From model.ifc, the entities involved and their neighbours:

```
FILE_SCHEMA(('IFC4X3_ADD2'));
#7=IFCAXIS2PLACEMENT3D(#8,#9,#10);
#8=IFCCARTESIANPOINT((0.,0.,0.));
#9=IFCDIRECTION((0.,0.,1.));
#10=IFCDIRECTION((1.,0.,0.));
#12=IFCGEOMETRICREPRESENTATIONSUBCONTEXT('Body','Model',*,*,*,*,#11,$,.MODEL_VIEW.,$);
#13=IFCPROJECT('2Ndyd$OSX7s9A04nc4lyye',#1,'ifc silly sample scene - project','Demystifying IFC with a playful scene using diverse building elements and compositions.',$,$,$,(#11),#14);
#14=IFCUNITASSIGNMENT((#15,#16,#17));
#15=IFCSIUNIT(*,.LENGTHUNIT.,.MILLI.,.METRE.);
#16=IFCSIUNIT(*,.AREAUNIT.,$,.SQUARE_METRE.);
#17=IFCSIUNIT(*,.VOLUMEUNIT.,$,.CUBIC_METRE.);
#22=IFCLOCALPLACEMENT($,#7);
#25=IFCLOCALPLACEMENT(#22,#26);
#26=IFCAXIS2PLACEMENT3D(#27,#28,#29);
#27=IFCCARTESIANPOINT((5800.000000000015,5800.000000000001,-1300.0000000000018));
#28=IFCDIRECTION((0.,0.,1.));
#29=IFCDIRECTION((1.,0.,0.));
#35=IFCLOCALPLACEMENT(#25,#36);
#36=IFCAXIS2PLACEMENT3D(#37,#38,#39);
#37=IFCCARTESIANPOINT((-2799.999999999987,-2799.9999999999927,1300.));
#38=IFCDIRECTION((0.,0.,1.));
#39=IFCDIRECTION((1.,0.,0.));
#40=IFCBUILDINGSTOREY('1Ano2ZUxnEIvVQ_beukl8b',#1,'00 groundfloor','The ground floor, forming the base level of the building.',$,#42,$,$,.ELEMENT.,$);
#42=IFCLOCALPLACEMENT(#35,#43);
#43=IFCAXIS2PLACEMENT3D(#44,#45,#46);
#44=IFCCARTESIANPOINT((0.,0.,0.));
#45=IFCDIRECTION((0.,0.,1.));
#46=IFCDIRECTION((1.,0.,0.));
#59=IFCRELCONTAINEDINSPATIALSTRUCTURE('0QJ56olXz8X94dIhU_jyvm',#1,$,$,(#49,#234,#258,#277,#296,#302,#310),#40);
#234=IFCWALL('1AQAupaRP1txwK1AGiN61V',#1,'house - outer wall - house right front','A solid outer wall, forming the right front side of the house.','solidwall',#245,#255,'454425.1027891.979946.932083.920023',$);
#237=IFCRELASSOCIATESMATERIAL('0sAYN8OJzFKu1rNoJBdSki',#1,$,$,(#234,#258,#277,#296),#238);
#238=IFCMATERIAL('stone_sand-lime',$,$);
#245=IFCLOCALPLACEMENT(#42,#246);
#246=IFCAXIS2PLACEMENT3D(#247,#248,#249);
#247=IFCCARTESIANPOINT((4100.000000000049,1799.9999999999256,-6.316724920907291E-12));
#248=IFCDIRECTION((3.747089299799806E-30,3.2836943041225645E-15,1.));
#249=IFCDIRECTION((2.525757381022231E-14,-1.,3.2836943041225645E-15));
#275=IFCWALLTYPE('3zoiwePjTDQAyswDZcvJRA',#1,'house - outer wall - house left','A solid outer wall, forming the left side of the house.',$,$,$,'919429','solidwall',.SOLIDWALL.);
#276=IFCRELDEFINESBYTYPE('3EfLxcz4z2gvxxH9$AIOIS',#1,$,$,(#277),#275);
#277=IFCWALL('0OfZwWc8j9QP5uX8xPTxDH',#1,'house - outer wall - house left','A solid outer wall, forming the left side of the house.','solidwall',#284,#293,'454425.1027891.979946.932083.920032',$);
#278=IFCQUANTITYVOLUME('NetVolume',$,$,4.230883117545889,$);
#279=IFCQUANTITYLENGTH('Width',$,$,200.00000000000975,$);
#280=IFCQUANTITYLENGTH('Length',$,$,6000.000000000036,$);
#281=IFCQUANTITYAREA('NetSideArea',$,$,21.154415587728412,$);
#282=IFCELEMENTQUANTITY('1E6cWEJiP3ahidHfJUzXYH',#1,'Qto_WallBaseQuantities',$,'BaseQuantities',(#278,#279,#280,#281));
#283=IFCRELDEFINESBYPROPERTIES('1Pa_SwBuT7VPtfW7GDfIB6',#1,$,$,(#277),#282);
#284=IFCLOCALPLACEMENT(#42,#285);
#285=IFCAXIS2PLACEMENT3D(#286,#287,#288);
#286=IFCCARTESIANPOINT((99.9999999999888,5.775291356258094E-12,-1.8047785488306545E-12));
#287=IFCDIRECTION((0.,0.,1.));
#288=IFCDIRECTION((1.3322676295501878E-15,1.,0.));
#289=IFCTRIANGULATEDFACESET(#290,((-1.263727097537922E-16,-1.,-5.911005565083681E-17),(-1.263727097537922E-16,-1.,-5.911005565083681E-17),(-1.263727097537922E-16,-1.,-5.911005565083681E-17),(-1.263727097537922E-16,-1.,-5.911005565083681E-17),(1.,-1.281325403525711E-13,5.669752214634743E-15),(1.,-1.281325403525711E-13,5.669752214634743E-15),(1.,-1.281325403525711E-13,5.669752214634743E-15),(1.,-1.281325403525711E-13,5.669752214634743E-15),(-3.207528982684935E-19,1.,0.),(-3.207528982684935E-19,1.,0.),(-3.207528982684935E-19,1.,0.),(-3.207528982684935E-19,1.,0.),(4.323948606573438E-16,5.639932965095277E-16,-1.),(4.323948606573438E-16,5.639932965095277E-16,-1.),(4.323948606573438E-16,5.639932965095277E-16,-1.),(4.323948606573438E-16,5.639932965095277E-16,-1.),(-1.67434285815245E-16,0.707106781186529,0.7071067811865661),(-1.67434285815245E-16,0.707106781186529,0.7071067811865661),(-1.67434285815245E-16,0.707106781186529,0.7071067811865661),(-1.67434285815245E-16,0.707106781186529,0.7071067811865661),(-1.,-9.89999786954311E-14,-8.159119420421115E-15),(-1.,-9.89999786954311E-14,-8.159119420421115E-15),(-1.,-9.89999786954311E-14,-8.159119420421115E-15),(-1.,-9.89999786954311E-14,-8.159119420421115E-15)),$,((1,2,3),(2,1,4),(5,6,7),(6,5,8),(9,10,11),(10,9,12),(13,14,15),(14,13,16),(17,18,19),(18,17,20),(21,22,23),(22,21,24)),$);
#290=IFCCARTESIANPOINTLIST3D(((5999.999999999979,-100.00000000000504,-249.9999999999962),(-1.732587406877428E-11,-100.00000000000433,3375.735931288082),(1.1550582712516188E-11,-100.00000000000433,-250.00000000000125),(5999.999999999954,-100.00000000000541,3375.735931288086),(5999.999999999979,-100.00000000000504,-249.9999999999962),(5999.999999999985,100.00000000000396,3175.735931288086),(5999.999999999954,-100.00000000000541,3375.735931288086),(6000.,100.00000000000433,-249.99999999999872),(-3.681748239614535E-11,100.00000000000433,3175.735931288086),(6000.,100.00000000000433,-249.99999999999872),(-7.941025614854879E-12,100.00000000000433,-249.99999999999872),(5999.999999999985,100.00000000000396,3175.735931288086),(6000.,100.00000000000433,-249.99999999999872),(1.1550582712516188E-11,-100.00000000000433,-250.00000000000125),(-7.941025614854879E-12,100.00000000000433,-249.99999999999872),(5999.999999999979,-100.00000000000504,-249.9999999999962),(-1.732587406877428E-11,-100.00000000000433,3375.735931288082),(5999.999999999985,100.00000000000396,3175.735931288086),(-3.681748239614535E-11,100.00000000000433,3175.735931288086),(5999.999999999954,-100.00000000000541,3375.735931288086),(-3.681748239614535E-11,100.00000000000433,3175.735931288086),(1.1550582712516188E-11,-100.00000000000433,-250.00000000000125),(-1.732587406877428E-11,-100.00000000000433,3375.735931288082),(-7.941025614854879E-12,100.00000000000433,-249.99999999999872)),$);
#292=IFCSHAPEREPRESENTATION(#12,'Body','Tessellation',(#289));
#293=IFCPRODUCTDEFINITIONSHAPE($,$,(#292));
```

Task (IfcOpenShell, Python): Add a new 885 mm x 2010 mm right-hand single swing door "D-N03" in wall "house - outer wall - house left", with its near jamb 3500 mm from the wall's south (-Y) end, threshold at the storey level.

```python
import numpy as np
import ifcopenshell
import ifcopenshell.api.feature
import ifcopenshell.api.geometry
import ifcopenshell.api.pset
import ifcopenshell.api.root
import ifcopenshell.api.spatial
import ifcopenshell.geom
import ifcopenshell.util.element
import ifcopenshell.util.placement
import ifcopenshell.util.representation
import ifcopenshell.util.shape
import ifcopenshell.util.unit

model = ifcopenshell.open("model.ifc")
unit_scale = ifcopenshell.util.unit.calculate_unit_scale(model)
area_scale = ifcopenshell.util.unit.calculate_unit_scale(model, "AREAUNIT")
volume_scale = ifcopenshell.util.unit.calculate_unit_scale(model, "VOLUMEUNIT")
settings = ifcopenshell.geom.settings()


def volume(element):
    """Net volume in cubic metres, openings subtracted."""
    shape = ifcopenshell.geom.create_shape(settings, element)
    return ifcopenshell.util.shape.get_volume(shape.geometry)


wall = model.by_guid("0OfZwWc8j9QP5uX8xPTxDH")
storey = ifcopenshell.util.element.get_container(wall, ifc_class="IfcBuildingStorey")
context = ifcopenshell.util.representation.get_context(model, "Model", "Body", "MODEL_VIEW")
before = volume(wall)

width, height, from_end, sill = 0.885, 2.01, 3.5, 0.0  # metres

# The wall runs along its own X axis, and the end named is its -X end.
wall_shape = ifcopenshell.geom.create_shape(settings, wall)
x, y, z = ifcopenshell.util.shape.get_vertices(wall_shape.geometry).T
start = x.min() + from_end
face, thickness = float(y.min()), float(y.max() - y.min())
wall_matrix = ifcopenshell.util.placement.get_local_placement(wall.ObjectPlacement)
level = ifcopenshell.util.placement.get_local_placement(storey.ObjectPlacement)[2, 3]


def in_wall(x, y):
    """Placement at x, y metres in the wall's axes, at sill height."""
    matrix = wall_matrix.copy()
    matrix[:, 3] = wall_matrix @ np.array([x / unit_scale, y / unit_scale, 0.0, 1.0])
    matrix[2, 3] = level + sill / unit_scale
    return matrix


# Opening: a box that overshoots both wall faces by 50 mm.
opening = ifcopenshell.api.root.create_entity(model, ifc_class="IfcOpeningElement", predefined_type="OPENING")
box = ifcopenshell.api.geometry.add_wall_representation(
    model, context=context, length=width, height=height, thickness=thickness + 0.1
)
ifcopenshell.api.geometry.assign_representation(model, product=opening, representation=box)
ifcopenshell.api.geometry.edit_object_placement(model, product=opening, matrix=in_wall(start, face - 0.05), is_si=False)
ifcopenshell.api.feature.add_feature(model, feature=opening, element=wall)

door = ifcopenshell.api.root.create_entity(model, ifc_class="IfcDoor", name="D-N03", predefined_type="DOOR")
door.OverallWidth, door.OverallHeight = width / unit_scale, height / unit_scale
door.OperationType = "SINGLE_SWING_RIGHT"
body = ifcopenshell.api.geometry.add_door_representation(
    model,
    context=context,
    overall_width=door.OverallWidth,
    overall_height=door.OverallHeight,
    operation_type="SINGLE_SWING_RIGHT",
    lining_properties={"LiningDepth": thickness / unit_scale, "ThresholdDepth": thickness / unit_scale},
)
ifcopenshell.api.geometry.assign_representation(model, product=door, representation=body)
ifcopenshell.api.spatial.assign_container(model, products=[door], relating_structure=storey)
ifcopenshell.api.feature.add_filling(model, opening=opening, element=door)

# The lining spans the wall, so the door starts at the wall face.
ifcopenshell.api.geometry.edit_object_placement(model, product=door, matrix=in_wall(start, face), is_si=False)

after = volume(wall)

# Update the wall's stored quantities.
qto = model.by_id(ifcopenshell.util.element.get_pset(wall, "Qto_WallBaseQuantities", should_inherit=False)["id"])
ifcopenshell.api.pset.edit_qto(model, qto=qto, properties={
    "NetVolume": after / volume_scale,
    "NetSideArea": after / thickness / area_scale,
})

print(f"wall volume {before:.3f} -> {after:.3f} m3")

model.write("model-out.ifc")
```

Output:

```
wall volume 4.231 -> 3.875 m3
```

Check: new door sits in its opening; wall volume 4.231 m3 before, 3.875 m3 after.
